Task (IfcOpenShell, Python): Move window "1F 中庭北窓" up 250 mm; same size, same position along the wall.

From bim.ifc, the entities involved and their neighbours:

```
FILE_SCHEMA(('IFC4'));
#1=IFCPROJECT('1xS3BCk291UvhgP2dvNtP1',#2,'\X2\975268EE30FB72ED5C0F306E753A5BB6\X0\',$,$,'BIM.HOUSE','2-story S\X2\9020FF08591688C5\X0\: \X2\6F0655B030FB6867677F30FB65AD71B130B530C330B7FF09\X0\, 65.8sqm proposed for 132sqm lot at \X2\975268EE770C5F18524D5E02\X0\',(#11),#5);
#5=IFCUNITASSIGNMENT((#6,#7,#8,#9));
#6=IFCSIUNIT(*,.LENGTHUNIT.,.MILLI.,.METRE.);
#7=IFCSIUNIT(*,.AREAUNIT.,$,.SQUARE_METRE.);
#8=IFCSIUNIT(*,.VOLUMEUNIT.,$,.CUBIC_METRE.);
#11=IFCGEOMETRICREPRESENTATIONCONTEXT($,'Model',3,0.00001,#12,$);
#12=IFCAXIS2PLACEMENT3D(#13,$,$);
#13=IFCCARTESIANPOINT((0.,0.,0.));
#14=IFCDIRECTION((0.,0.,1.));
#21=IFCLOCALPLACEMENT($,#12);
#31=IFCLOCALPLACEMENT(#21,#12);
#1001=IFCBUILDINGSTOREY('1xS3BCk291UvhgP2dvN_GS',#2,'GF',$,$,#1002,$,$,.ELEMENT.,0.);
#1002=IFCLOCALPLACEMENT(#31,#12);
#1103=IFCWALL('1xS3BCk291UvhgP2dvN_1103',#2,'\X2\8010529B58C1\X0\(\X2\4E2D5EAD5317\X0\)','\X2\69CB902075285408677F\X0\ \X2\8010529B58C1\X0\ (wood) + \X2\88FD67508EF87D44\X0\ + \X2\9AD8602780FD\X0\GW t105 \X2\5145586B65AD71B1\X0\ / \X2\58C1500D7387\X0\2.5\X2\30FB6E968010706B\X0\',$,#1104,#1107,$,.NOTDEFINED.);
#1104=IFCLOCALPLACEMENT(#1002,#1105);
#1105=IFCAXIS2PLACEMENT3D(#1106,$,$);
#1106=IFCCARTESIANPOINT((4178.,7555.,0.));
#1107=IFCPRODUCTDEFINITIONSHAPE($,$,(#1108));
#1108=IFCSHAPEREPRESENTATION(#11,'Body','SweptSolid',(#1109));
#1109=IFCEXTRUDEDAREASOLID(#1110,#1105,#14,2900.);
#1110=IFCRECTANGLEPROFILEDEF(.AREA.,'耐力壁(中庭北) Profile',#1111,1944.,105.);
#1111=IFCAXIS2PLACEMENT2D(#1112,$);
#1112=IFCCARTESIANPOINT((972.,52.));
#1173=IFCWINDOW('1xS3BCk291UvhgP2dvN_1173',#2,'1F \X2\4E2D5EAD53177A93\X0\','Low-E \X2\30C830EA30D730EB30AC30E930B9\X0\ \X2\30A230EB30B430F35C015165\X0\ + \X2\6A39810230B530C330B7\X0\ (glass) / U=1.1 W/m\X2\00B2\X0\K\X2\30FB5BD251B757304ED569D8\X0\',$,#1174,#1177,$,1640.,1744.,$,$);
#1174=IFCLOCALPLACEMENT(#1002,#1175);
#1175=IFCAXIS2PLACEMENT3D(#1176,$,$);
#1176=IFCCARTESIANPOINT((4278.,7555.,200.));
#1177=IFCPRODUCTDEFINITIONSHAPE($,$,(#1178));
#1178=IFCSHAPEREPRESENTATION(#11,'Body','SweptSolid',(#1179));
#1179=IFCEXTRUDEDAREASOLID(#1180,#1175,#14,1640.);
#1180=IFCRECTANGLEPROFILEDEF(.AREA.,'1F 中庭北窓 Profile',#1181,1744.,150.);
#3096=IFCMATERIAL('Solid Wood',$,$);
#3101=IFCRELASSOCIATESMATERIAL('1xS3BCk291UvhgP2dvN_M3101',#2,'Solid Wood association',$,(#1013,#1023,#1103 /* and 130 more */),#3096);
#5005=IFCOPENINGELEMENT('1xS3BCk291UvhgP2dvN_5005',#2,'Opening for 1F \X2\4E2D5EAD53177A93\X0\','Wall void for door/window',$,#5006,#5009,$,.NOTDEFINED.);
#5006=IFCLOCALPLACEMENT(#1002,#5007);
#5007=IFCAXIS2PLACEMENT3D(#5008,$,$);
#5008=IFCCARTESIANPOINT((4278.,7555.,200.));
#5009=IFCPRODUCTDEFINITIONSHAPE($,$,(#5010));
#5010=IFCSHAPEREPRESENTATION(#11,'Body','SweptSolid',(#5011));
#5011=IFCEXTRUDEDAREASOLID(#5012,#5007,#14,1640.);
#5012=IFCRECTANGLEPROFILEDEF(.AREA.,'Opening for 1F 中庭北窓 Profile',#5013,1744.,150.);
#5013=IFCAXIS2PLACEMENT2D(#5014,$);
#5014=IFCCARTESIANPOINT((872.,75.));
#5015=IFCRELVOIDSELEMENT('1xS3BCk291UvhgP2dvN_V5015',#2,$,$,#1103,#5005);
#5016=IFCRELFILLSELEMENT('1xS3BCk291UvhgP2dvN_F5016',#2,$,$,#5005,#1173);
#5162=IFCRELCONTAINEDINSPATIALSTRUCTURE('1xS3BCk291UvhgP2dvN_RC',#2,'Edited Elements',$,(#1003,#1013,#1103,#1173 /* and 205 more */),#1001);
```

```python
import numpy as np
import ifcopenshell
import ifcopenshell.api.geometry
import ifcopenshell.util.placement
import ifcopenshell.util.unit

model = ifcopenshell.open("bim.ifc")
unit_scale = ifcopenshell.util.unit.calculate_unit_scale(model)

window = model.by_id(1173)
opening = window.FillsVoids[0].RelatingOpeningElement
dz = 0.25 / unit_scale

shift = np.array([0.0, 0.0, dz])
# The window is not placed relative to its opening, so move both.
for product in (opening, window):
    matrix = ifcopenshell.util.placement.get_local_placement(product.ObjectPlacement)
    matrix[:3, 3] += shift
    ifcopenshell.api.geometry.edit_object_placement(model, product=product, matrix=matrix, is_si=False)

print(f"moved by {dz * unit_scale:+.3f} m")

model.write("bim_v2.ifc")
```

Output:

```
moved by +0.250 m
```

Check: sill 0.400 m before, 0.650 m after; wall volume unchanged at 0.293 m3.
